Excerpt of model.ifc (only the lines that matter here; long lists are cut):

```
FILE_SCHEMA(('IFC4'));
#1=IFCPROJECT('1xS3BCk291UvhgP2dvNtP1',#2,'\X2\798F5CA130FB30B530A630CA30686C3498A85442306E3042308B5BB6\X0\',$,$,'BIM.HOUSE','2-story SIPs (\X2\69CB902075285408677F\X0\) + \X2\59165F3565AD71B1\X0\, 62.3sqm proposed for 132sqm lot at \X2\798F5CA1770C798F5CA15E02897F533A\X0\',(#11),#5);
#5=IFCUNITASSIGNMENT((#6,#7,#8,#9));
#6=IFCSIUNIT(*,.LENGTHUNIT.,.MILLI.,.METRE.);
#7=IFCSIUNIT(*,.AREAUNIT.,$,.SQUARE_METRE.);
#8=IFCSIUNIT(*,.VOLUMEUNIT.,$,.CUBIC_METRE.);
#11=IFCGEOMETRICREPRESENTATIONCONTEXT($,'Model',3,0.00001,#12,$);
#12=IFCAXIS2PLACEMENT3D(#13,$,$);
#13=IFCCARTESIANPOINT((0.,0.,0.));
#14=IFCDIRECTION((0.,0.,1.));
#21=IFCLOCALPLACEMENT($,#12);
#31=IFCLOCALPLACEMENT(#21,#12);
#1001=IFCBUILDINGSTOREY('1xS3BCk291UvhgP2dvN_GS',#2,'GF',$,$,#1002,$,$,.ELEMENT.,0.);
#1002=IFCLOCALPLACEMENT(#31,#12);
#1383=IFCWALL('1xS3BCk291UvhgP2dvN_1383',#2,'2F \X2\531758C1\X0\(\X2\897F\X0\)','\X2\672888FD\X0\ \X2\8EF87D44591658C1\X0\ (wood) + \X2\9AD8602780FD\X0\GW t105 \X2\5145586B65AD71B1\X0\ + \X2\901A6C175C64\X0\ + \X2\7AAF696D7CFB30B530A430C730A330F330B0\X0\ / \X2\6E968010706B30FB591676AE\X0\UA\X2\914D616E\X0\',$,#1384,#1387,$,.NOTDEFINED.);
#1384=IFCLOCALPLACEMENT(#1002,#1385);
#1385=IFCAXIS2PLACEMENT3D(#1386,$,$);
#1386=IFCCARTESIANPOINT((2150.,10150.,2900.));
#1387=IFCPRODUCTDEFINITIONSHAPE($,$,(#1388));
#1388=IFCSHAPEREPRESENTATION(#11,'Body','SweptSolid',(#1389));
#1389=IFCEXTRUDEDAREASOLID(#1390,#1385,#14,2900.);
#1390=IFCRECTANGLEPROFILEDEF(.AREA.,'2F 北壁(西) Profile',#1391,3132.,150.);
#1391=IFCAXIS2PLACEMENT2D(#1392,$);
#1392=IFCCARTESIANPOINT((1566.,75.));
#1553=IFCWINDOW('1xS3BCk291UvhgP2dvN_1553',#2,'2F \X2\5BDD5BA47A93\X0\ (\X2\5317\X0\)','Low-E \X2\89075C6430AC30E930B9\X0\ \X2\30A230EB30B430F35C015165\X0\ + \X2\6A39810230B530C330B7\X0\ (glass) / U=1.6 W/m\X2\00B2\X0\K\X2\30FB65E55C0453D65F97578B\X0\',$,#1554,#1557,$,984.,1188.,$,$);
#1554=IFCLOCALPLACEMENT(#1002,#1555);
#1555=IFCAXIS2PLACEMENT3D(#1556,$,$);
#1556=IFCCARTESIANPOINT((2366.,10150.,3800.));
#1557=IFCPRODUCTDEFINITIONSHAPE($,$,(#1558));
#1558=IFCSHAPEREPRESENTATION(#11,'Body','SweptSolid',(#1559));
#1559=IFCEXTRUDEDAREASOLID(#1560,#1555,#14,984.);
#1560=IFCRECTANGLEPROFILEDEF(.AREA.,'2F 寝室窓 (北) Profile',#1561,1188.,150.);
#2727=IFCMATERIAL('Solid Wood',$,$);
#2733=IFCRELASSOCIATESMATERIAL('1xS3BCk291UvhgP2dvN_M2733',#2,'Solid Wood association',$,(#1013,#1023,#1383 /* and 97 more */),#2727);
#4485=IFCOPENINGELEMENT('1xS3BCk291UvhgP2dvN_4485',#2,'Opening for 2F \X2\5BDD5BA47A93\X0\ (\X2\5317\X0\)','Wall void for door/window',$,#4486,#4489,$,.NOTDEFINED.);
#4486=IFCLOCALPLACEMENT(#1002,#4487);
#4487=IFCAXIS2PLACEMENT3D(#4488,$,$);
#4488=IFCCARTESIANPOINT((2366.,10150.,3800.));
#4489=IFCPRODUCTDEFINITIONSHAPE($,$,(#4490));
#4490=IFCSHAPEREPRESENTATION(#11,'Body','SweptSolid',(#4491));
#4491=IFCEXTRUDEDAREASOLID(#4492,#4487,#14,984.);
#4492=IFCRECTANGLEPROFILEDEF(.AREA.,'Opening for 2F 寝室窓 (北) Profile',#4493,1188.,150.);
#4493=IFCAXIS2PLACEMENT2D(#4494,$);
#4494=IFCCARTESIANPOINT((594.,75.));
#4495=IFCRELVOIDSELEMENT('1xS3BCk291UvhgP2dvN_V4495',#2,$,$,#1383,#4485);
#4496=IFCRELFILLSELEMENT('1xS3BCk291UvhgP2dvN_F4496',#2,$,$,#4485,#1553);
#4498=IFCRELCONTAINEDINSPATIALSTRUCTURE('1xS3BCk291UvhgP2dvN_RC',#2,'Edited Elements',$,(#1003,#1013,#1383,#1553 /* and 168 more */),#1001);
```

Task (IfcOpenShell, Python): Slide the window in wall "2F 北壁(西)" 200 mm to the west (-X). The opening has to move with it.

```python
import ifcopenshell
import ifcopenshell.api.geometry
import ifcopenshell.util.placement

model = ifcopenshell.open("model.ifc")

window = model.by_guid("1xS3BCk291UvhgP2dvN_1553")
opening = window.FillsVoids[0].RelatingOpeningElement
wall = opening.VoidsElements[0].RelatingBuildingElement

wall_matrix = ifcopenshell.util.placement.get_local_placement(wall.ObjectPlacement)
shift = wall_matrix[:3, 0] * -200.0
before = ifcopenshell.util.placement.get_local_placement(window.ObjectPlacement)[:3, 3].copy()

# The window is not placed relative to its opening, so move both.
for product in (opening, window):
    matrix = ifcopenshell.util.placement.get_local_placement(product.ObjectPlacement)
    matrix[:3, 3] += shift
    ifcopenshell.api.geometry.edit_object_placement(model, product=product, matrix=matrix, is_si=False)

after = ifcopenshell.util.placement.get_local_placement(window.ObjectPlacement)[:3, 3]
print("window moved by", (after - before).round(3) + 0.0)

model.write("model_rev.ifc")
```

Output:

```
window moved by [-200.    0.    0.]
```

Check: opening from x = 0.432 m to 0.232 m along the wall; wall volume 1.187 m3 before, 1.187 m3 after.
